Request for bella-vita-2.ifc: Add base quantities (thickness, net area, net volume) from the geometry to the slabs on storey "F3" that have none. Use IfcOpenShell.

First a look at what the model holds.

```python
import ifcopenshell
import ifcopenshell.util.element
import ifcopenshell.util.unit

model = ifcopenshell.open("bella-vita-2.ifc")
print(model.schema)
for unit_type in ("LENGTHUNIT", "AREAUNIT", "VOLUMEUNIT"):
    print(unit_type, ifcopenshell.util.unit.calculate_unit_scale(model, unit_type))
storey = next(s for s in model.by_type("IfcBuildingStorey") if s.Name == "F3")
slabs = [e for e in ifcopenshell.util.element.get_decomposition(storey) if e.is_a("IfcSlab")]
for e in sorted(slabs, key=lambda e: e.id()):
    print(e.id(), e.is_a(), e.Name, list(ifcopenshell.util.element.get_psets(e, qtos_only=True)), sep=" | ")
```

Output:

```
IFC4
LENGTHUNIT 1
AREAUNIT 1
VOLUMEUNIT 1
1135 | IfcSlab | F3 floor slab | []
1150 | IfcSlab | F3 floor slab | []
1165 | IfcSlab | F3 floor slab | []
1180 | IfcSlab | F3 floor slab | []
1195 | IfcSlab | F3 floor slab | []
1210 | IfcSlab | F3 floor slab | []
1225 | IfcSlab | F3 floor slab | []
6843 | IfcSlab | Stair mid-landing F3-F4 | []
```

```python
import ifcopenshell
import ifcopenshell.api.pset
import ifcopenshell.geom
import ifcopenshell.util.element
import ifcopenshell.util.shape
import ifcopenshell.util.unit

model = ifcopenshell.open("bella-vita-2.ifc")
unit_scale = ifcopenshell.util.unit.calculate_unit_scale(model)
area_scale = ifcopenshell.util.unit.calculate_unit_scale(model, "AREAUNIT")
volume_scale = ifcopenshell.util.unit.calculate_unit_scale(model, "VOLUMEUNIT")
settings = ifcopenshell.geom.settings()

storey = next(s for s in model.by_type("IfcBuildingStorey") if s.Name == "F3")
slabs = [e for e in ifcopenshell.util.element.get_decomposition(storey) if e.is_a("IfcSlab")]

for e in sorted(slabs, key=lambda e: e.id()):
    if ifcopenshell.util.element.get_psets(e, qtos_only=True, should_inherit=False):
        continue
    # Geometry comes back in metres, in the element's own axes.
    shape = ifcopenshell.geom.create_shape(settings, e)
    values = {
        "Width": ifcopenshell.util.shape.get_z(shape.geometry) / unit_scale,
        "NetArea": ifcopenshell.util.shape.get_footprint_area(shape.geometry) / area_scale,
        "NetVolume": ifcopenshell.util.shape.get_volume(shape.geometry) / volume_scale,
    }
    qto = ifcopenshell.api.pset.add_qto(model, product=e, name="Qto_SlabBaseQuantities")
    ifcopenshell.api.pset.edit_qto(model, qto=qto, properties=values)
    print(e.id(), {k: round(v, 3) for k, v in values.items()})

model.write("bella-vita-2_rev.ifc")
```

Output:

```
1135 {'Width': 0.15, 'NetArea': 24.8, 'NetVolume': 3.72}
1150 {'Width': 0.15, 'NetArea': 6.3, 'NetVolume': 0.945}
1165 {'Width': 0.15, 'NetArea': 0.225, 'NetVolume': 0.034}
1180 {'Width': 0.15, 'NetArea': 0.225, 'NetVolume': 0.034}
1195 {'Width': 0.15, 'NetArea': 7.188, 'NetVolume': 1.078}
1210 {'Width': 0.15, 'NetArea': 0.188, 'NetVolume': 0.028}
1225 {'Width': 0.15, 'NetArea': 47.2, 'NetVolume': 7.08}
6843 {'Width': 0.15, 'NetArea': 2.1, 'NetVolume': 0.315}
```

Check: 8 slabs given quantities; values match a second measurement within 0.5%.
